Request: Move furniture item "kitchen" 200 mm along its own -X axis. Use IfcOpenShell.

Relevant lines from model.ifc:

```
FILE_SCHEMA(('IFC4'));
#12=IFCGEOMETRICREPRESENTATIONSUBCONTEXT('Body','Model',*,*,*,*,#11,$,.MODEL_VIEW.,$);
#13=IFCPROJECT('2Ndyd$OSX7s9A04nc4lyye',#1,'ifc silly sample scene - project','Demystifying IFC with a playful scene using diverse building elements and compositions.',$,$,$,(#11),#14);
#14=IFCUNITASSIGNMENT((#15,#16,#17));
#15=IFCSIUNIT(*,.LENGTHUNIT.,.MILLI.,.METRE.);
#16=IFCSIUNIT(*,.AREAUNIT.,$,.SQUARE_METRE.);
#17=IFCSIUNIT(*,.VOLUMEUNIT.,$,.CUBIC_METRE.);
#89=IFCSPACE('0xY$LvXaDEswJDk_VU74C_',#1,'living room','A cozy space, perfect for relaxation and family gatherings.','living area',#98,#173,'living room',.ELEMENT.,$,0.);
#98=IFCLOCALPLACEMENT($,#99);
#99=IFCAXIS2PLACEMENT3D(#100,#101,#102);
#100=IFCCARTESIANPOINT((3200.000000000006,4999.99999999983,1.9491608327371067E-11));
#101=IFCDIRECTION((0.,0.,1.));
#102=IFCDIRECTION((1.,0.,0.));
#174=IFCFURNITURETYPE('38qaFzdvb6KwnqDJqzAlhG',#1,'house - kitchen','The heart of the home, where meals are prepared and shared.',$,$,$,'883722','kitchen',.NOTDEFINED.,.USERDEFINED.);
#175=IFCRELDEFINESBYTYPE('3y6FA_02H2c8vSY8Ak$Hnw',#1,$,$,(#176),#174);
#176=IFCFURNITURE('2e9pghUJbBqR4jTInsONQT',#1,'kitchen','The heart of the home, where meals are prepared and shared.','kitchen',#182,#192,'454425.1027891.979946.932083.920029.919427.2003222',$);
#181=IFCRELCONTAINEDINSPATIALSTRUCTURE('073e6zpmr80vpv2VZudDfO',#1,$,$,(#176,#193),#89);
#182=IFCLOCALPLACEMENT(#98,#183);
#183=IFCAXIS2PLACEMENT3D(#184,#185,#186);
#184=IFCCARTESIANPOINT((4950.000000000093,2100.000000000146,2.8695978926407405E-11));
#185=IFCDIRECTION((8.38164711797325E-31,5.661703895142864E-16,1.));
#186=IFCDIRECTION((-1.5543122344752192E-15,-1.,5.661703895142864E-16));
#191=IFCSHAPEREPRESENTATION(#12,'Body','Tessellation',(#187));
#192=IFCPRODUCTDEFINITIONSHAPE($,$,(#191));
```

```python
import ifcopenshell
import ifcopenshell.api.geometry
import ifcopenshell.util.placement
import ifcopenshell.util.unit

model = ifcopenshell.open("model.ifc")
unit_scale = ifcopenshell.util.unit.calculate_unit_scale(model)

item = model.by_guid("2e9pghUJbBqR4jTInsONQT")
matrix = ifcopenshell.util.placement.get_local_placement(item.ObjectPlacement)
matrix[:3, 3] -= matrix[:3, 0] * 0.2 / unit_scale
ifcopenshell.api.geometry.edit_object_placement(model, product=item, matrix=matrix, is_si=False)

print(ifcopenshell.util.placement.get_local_placement(item.ObjectPlacement).round(3) + 0.0)

model.write("model_edited.ifc")
```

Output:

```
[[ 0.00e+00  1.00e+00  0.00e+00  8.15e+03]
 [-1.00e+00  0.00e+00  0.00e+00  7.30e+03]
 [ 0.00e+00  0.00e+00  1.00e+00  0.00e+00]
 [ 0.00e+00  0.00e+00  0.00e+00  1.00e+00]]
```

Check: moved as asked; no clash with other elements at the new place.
